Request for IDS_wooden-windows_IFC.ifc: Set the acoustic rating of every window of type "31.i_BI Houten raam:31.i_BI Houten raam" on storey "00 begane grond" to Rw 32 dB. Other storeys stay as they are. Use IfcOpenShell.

First a look at what the model holds.

```python
import ifcopenshell
import ifcopenshell.util.element

model = ifcopenshell.open("IDS_wooden-windows_IFC.ifc")
print(model.schema)
storey = next(s for s in model.by_type("IfcBuildingStorey") if s.Name == "00 begane grond")
windows = [e for e in ifcopenshell.util.element.get_decomposition(storey) if e.is_a("IfcWindow")]
seen = {}
for e in windows:
    element_type = ifcopenshell.util.element.get_type(e)
    key = (element_type.Name if element_type != e and element_type else None, ifcopenshell.util.element.get_pset(e, "Pset_WindowCommon", "AcousticRating"))
    seen[key] = seen.get(key, 0) + 1
for (name, value), count in sorted(seen.items(), key=str):
    print(count, "x", name, "|", value)
```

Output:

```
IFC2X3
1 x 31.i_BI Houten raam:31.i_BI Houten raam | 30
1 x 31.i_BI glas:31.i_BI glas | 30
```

```python
import ifcopenshell
import ifcopenshell.api.pset
import ifcopenshell.util.element

model = ifcopenshell.open("IDS_wooden-windows_IFC.ifc")

storey = next(s for s in model.by_type("IfcBuildingStorey") if s.Name == "00 begane grond")
windows = [e for e in ifcopenshell.util.element.get_decomposition(storey) if e.is_a("IfcWindow")]

count = 0
for e in windows:
    element_type = ifcopenshell.util.element.get_type(e)
    if element_type in (None, e) or element_type.Name != "31.i_BI Houten raam:31.i_BI Houten raam":
        continue
    # add_pset returns the element's existing set when there is one.
    pset = ifcopenshell.api.pset.add_pset(model, product=e, name="Pset_WindowCommon")
    ifcopenshell.api.pset.edit_pset(model, pset=pset, properties={"AcousticRating": "Rw 32 dB"})
    count += 1

print(count, "windows updated")

model.write("IDS_wooden-windows_IFC_rev.ifc")
```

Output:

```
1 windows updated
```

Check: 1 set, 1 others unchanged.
